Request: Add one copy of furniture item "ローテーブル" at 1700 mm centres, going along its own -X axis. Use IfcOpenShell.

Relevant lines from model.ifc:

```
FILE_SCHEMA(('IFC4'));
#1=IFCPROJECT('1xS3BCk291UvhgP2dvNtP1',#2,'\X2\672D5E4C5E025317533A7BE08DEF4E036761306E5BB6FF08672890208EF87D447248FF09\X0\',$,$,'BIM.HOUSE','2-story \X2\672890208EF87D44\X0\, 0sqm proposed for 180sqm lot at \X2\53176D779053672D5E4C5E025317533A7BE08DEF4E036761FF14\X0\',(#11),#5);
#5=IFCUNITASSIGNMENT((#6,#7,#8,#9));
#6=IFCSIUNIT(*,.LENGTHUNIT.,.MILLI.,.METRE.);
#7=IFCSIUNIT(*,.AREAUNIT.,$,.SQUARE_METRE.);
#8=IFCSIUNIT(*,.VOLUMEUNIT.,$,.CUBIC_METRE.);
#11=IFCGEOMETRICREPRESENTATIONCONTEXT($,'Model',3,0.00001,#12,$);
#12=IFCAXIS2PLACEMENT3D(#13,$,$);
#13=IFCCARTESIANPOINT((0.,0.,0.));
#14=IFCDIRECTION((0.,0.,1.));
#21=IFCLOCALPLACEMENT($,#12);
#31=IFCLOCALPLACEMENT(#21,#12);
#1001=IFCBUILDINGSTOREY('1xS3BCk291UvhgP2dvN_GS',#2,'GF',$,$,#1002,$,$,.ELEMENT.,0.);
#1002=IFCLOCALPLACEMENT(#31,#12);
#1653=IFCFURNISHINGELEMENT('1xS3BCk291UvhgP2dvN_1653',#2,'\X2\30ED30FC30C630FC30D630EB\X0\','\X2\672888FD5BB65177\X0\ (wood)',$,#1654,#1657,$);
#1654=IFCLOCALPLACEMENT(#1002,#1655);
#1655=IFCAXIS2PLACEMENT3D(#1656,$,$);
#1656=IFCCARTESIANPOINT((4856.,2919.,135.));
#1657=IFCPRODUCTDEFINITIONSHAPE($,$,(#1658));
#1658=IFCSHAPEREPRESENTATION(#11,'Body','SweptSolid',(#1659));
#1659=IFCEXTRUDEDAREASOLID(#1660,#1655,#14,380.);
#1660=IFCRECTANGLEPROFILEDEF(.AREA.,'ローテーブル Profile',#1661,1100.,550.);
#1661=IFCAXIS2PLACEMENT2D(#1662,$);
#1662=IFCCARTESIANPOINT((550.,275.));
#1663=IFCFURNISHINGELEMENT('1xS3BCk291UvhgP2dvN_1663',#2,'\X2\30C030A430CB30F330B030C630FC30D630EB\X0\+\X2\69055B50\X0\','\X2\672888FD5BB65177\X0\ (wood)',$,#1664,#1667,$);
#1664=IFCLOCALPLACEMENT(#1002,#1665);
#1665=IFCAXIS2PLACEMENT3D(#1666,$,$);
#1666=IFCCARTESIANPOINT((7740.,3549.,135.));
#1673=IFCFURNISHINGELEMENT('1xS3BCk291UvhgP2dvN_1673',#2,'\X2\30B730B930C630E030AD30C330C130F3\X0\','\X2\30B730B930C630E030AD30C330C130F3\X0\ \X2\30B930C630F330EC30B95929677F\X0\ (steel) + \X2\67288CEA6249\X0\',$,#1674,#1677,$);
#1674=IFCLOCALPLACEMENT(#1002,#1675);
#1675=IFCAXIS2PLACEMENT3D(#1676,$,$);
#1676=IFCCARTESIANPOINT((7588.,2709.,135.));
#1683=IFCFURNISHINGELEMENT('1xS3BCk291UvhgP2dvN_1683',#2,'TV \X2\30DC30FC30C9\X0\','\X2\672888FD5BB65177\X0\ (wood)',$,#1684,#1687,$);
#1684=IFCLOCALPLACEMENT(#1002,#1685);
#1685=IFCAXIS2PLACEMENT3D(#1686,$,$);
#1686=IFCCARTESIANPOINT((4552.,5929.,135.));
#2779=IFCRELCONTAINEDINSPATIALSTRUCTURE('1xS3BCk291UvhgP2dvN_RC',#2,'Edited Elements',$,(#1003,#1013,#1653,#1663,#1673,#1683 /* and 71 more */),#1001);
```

```python
import ifcopenshell
import ifcopenshell.api.geometry
import ifcopenshell.api.root
import ifcopenshell.util.element
import ifcopenshell.util.placement
import ifcopenshell.util.unit

model = ifcopenshell.open("model.ifc")
unit_scale = ifcopenshell.util.unit.calculate_unit_scale(model)


def reuse_history(source, copy):
    """copy_class also copies each property set's owner history, people and application; keep the originals."""
    for rel in copy.IsDefinedBy:
        if rel.is_a("IfcRelDefinesByProperties") and (history := rel.RelatingPropertyDefinition.OwnerHistory):
            rel.RelatingPropertyDefinition.OwnerHistory = source.OwnerHistory
            ifcopenshell.util.element.remove_deep2(model, history)


source = model.by_guid("1xS3BCk291UvhgP2dvN_1653")
base = ifcopenshell.util.placement.get_local_placement(source.ObjectPlacement)
step = -base[:3, 0] * 1.7 / unit_scale

for i in range(1, 2):
    copy = ifcopenshell.api.root.copy_class(model, product=source)
    copy.Representation = ifcopenshell.util.element.copy_deep(
        model, source.Representation, exclude=["IfcGeometricRepresentationContext", "IfcRepresentationMap"]
    )
    reuse_history(source, copy)
    matrix = base.copy()
    matrix[:3, 3] += i * step
    print("added at", matrix[:3, 3].round(3) + 0.0)
    ifcopenshell.api.geometry.edit_object_placement(model, product=copy, matrix=matrix, is_si=False)

model.write("model_edited.ifc")
```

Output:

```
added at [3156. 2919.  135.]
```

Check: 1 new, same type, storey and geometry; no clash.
